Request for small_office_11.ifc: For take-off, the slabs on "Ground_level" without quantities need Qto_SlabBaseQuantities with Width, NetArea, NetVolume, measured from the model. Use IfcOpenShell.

First a look at what the model holds.

```python
import ifcopenshell
import ifcopenshell.util.element
import ifcopenshell.util.unit

model = ifcopenshell.open("small_office_11.ifc")
print(model.schema)
for unit_type in ("LENGTHUNIT", "AREAUNIT", "VOLUMEUNIT"):
    print(unit_type, ifcopenshell.util.unit.calculate_unit_scale(model, unit_type))
storey = next(s for s in model.by_type("IfcBuildingStorey") if s.Name == "Ground_level")
slabs = [e for e in ifcopenshell.util.element.get_decomposition(storey) if e.is_a("IfcSlab")]
for e in sorted(slabs, key=lambda e: e.id()):
    print(e.id(), e.is_a(), e.Name, list(ifcopenshell.util.element.get_psets(e, qtos_only=True)), sep=" | ")
```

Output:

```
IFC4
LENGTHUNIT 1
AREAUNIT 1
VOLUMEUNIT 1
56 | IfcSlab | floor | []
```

```python
import ifcopenshell
import ifcopenshell.api.pset
import ifcopenshell.geom
import ifcopenshell.util.element
import ifcopenshell.util.shape
import ifcopenshell.util.unit

model = ifcopenshell.open("small_office_11.ifc")
unit_scale = ifcopenshell.util.unit.calculate_unit_scale(model)
area_scale = ifcopenshell.util.unit.calculate_unit_scale(model, "AREAUNIT")
volume_scale = ifcopenshell.util.unit.calculate_unit_scale(model, "VOLUMEUNIT")
settings = ifcopenshell.geom.settings()

storey = next(s for s in model.by_type("IfcBuildingStorey") if s.Name == "Ground_level")
slabs = [e for e in ifcopenshell.util.element.get_decomposition(storey) if e.is_a("IfcSlab")]

for e in sorted(slabs, key=lambda e: e.id()):
    if ifcopenshell.util.element.get_psets(e, qtos_only=True, should_inherit=False):
        continue
    # Geometry comes back in metres, in the element's own axes.
    shape = ifcopenshell.geom.create_shape(settings, e)
    values = {
        "Width": ifcopenshell.util.shape.get_z(shape.geometry) / unit_scale,
        "NetArea": ifcopenshell.util.shape.get_footprint_area(shape.geometry) / area_scale,
        "NetVolume": ifcopenshell.util.shape.get_volume(shape.geometry) / volume_scale,
    }
    qto = ifcopenshell.api.pset.add_qto(model, product=e, name="Qto_SlabBaseQuantities")
    ifcopenshell.api.pset.edit_qto(model, qto=qto, properties=values)
    print(e.id(), {k: round(v, 3) for k, v in values.items()})

model.write("small_office_11_updated.ifc")
```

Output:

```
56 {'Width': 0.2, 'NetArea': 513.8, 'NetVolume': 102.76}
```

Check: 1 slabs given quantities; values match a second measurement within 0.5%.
